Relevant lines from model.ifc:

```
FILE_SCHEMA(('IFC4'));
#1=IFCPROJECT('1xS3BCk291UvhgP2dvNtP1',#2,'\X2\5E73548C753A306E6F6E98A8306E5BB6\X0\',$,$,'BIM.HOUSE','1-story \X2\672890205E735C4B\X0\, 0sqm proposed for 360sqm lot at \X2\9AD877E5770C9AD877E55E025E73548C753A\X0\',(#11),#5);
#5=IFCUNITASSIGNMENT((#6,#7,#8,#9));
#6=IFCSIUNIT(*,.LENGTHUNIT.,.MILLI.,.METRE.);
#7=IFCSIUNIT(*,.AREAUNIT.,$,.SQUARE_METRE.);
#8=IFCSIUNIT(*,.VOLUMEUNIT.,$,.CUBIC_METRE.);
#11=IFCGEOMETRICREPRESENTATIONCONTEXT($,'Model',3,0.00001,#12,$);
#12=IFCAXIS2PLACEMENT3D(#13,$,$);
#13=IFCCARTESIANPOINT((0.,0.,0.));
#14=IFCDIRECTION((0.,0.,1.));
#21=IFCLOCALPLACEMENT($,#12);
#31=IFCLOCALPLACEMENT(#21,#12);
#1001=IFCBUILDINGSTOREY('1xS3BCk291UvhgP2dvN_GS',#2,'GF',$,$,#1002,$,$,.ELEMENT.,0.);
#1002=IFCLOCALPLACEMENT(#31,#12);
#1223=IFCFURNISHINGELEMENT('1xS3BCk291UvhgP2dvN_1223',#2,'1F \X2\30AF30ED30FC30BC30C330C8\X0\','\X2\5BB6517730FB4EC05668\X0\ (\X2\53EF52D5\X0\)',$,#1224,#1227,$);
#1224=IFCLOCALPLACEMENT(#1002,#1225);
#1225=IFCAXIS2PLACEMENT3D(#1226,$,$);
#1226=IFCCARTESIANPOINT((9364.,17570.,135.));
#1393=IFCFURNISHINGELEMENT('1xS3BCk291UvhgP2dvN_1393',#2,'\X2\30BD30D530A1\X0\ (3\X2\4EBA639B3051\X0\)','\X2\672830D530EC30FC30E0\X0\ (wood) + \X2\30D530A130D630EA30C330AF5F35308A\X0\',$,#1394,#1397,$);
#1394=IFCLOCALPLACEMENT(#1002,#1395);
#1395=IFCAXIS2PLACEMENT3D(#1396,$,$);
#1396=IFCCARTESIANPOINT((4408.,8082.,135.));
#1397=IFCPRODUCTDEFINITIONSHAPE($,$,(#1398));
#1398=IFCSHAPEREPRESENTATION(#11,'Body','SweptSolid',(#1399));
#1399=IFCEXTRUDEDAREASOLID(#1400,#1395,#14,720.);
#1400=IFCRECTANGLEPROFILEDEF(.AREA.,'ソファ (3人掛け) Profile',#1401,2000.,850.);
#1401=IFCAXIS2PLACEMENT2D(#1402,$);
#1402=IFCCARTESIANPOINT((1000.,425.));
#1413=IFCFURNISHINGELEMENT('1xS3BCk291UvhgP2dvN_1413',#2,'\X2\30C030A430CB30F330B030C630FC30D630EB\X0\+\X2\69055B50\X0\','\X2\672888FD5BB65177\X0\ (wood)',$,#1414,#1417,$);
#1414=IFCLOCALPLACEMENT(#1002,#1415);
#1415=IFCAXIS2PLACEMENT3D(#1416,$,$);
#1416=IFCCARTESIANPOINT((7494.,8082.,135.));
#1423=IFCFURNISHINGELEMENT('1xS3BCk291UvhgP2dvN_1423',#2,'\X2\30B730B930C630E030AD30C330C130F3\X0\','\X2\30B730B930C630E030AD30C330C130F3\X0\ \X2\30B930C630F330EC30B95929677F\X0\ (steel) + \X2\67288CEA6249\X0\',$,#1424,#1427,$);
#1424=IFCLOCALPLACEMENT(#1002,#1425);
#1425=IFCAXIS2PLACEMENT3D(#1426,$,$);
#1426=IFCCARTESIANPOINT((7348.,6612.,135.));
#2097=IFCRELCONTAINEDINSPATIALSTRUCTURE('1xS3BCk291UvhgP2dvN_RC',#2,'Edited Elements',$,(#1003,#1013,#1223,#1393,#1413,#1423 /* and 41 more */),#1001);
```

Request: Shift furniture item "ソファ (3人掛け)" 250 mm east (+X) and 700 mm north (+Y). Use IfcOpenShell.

```python
import ifcopenshell
import ifcopenshell.api.geometry
import ifcopenshell.util.placement
import ifcopenshell.util.unit

model = ifcopenshell.open("model.ifc")
unit_scale = ifcopenshell.util.unit.calculate_unit_scale(model)

item = model.by_guid("1xS3BCk291UvhgP2dvN_1393")
matrix = ifcopenshell.util.placement.get_local_placement(item.ObjectPlacement)
matrix[0, 3] += 0.25 / unit_scale
matrix[1, 3] += 0.7 / unit_scale
ifcopenshell.api.geometry.edit_object_placement(model, product=item, matrix=matrix, is_si=False)

print(ifcopenshell.util.placement.get_local_placement(item.ObjectPlacement).round(3) + 0.0)

model.write("model-out.ifc")
```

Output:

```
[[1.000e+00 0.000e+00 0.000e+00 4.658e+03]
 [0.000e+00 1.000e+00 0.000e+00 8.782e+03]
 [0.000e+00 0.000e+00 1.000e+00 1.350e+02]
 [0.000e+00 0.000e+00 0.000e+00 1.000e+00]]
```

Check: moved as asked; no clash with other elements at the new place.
